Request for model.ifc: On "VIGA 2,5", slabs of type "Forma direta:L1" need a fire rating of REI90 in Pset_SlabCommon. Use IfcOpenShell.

First a look at what the model holds.

```python
import ifcopenshell
import ifcopenshell.util.element

model = ifcopenshell.open("model.ifc")
print(model.schema)
storey = next(s for s in model.by_type("IfcBuildingStorey") if s.Name == "VIGA 2,5")
slabs = [e for e in ifcopenshell.util.element.get_decomposition(storey) if e.is_a("IfcSlab")]
seen = {}
for e in slabs:
    element_type = ifcopenshell.util.element.get_type(e)
    key = (element_type.Name if element_type != e and element_type else None, ifcopenshell.util.element.get_pset(e, "Pset_SlabCommon", "FireRating"))
    seen[key] = seen.get(key, 0) + 1
for (name, value), count in sorted(seen.items(), key=str):
    print(count, "x", name, "|", value)
```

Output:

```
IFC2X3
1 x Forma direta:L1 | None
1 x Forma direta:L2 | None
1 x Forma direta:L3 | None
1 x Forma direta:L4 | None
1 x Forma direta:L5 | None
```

```python
import ifcopenshell
import ifcopenshell.api.pset
import ifcopenshell.util.element

model = ifcopenshell.open("model.ifc")

storey = next(s for s in model.by_type("IfcBuildingStorey") if s.Name == "VIGA 2,5")
slabs = [e for e in ifcopenshell.util.element.get_decomposition(storey) if e.is_a("IfcSlab")]

count = 0
for e in slabs:
    element_type = ifcopenshell.util.element.get_type(e)
    if element_type in (None, e) or element_type.Name != "Forma direta:L1":
        continue
    # add_pset returns the element's existing set when there is one.
    pset = ifcopenshell.api.pset.add_pset(model, product=e, name="Pset_SlabCommon")
    ifcopenshell.api.pset.edit_pset(model, pset=pset, properties={"FireRating": "REI90"})
    count += 1

print(count, "slabs updated")

model.write("model-out.ifc")
```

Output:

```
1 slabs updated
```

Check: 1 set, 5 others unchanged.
